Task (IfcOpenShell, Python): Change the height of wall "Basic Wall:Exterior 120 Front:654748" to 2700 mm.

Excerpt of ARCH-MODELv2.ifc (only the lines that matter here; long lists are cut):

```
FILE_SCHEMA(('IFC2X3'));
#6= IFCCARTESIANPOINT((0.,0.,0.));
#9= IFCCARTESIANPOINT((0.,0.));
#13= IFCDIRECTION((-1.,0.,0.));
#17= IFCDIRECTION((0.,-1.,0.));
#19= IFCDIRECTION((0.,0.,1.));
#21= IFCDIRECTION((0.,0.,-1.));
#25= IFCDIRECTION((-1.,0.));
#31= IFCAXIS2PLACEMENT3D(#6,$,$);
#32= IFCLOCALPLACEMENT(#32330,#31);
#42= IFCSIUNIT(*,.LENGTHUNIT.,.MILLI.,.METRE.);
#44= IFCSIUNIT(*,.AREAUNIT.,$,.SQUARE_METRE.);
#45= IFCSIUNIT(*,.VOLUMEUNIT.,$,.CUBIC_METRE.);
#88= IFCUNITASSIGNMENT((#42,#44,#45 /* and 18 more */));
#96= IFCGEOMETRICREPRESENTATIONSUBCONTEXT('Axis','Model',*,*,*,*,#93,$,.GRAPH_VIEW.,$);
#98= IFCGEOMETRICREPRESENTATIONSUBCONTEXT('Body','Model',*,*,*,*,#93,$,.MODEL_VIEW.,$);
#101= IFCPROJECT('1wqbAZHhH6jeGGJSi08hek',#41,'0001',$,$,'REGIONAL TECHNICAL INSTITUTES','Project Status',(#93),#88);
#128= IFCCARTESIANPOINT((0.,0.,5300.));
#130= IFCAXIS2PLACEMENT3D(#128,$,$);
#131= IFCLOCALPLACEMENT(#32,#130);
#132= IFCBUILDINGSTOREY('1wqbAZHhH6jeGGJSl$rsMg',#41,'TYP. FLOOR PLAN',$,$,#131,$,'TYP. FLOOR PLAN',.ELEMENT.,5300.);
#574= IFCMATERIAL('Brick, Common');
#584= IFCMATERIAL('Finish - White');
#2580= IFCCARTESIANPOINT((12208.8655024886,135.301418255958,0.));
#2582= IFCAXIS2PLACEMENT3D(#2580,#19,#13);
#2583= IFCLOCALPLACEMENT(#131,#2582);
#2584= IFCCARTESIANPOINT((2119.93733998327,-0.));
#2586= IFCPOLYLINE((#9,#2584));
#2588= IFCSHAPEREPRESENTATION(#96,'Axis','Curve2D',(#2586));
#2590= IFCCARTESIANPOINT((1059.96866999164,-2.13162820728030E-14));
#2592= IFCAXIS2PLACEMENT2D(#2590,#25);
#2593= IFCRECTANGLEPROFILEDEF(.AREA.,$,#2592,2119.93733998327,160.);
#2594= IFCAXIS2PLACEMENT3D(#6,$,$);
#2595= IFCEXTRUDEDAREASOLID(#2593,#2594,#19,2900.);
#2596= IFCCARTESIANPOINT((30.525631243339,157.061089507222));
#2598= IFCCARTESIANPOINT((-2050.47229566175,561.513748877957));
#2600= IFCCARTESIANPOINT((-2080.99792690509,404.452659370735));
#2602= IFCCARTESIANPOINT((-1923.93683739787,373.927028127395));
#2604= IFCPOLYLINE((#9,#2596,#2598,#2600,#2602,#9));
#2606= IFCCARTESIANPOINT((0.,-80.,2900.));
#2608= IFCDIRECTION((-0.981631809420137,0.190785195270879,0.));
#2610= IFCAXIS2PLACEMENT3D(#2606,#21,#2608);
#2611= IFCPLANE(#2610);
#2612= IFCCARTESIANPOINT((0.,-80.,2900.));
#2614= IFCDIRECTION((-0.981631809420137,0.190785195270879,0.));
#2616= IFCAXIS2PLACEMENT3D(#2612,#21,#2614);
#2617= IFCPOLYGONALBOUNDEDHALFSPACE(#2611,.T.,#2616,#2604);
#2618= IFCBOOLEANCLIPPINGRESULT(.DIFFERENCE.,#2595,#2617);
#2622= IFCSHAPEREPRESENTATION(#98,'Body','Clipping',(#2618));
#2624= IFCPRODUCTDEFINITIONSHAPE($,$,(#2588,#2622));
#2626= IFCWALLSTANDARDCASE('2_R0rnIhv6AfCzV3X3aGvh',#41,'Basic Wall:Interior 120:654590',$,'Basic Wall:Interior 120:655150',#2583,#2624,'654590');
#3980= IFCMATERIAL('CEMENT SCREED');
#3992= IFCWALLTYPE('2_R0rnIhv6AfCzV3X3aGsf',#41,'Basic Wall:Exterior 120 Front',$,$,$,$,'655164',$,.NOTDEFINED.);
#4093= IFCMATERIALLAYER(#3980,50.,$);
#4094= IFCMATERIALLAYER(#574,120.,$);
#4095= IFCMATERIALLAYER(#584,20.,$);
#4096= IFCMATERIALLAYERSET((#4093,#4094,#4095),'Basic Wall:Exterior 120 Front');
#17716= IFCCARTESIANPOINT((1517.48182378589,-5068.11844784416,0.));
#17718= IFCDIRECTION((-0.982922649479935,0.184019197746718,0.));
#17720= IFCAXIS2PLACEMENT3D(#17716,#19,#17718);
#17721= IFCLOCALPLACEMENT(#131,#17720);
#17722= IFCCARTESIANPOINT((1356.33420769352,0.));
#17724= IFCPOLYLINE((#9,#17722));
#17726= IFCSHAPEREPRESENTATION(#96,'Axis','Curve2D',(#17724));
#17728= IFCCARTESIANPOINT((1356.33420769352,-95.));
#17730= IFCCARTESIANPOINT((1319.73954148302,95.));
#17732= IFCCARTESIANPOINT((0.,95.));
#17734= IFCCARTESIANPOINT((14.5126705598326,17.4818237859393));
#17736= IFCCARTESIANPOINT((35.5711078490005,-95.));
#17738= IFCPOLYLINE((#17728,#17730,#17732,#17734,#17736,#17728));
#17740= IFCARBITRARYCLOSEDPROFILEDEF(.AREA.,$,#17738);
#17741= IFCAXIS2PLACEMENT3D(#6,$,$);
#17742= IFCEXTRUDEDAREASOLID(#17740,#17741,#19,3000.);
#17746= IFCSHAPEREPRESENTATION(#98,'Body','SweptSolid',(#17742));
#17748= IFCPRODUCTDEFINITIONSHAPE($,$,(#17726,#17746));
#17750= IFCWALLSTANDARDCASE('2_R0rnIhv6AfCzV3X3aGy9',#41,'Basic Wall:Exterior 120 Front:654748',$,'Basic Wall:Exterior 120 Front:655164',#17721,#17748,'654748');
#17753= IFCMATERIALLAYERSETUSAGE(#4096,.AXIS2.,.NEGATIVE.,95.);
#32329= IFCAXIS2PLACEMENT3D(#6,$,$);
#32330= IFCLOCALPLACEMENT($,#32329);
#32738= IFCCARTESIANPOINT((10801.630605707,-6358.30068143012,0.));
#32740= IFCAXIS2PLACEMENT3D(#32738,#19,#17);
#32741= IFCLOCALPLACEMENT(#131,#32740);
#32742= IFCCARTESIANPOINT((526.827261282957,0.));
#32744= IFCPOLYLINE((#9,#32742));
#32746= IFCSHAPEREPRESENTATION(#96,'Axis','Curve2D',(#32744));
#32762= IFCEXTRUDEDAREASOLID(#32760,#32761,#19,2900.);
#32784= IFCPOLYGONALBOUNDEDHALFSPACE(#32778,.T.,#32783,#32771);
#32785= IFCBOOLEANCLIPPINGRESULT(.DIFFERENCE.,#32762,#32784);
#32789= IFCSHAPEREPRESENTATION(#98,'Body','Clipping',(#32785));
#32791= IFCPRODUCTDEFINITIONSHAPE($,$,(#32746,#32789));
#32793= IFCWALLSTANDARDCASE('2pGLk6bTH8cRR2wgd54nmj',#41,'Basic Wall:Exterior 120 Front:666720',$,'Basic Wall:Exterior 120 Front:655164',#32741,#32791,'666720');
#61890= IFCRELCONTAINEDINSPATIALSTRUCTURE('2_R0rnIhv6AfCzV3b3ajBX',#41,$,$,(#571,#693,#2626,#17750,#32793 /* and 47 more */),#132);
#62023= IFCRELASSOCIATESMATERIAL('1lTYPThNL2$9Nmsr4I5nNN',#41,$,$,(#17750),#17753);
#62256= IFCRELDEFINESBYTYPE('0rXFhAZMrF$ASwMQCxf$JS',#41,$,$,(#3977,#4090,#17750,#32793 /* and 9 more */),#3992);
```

```python
import ifcopenshell
import ifcopenshell.geom
import ifcopenshell.util.representation
import ifcopenshell.util.shape
import ifcopenshell.util.unit

model = ifcopenshell.open("ARCH-MODELv2.ifc")
unit_scale = ifcopenshell.util.unit.calculate_unit_scale(model)
settings = ifcopenshell.geom.settings()


def volume(element):
    """Net volume in cubic metres, openings subtracted."""
    shape = ifcopenshell.geom.create_shape(settings, element)
    return ifcopenshell.util.shape.get_volume(shape.geometry)


wall = model.by_guid("2_R0rnIhv6AfCzV3X3aGy9")
before = volume(wall)

body = ifcopenshell.util.representation.get_representation(wall, "Model", "Body")
solid = body.Items[0]
old_height = solid.Depth
solid.Depth = 2.7 / unit_scale
after = volume(wall)

print(f"height {old_height:g} -> {solid.Depth:g}, volume {before:.3f} -> {after:.3f} m3")

model.write("ARCH-MODELv2_updated.ifc")
```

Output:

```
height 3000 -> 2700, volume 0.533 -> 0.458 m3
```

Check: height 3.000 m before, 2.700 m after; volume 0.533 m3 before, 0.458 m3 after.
